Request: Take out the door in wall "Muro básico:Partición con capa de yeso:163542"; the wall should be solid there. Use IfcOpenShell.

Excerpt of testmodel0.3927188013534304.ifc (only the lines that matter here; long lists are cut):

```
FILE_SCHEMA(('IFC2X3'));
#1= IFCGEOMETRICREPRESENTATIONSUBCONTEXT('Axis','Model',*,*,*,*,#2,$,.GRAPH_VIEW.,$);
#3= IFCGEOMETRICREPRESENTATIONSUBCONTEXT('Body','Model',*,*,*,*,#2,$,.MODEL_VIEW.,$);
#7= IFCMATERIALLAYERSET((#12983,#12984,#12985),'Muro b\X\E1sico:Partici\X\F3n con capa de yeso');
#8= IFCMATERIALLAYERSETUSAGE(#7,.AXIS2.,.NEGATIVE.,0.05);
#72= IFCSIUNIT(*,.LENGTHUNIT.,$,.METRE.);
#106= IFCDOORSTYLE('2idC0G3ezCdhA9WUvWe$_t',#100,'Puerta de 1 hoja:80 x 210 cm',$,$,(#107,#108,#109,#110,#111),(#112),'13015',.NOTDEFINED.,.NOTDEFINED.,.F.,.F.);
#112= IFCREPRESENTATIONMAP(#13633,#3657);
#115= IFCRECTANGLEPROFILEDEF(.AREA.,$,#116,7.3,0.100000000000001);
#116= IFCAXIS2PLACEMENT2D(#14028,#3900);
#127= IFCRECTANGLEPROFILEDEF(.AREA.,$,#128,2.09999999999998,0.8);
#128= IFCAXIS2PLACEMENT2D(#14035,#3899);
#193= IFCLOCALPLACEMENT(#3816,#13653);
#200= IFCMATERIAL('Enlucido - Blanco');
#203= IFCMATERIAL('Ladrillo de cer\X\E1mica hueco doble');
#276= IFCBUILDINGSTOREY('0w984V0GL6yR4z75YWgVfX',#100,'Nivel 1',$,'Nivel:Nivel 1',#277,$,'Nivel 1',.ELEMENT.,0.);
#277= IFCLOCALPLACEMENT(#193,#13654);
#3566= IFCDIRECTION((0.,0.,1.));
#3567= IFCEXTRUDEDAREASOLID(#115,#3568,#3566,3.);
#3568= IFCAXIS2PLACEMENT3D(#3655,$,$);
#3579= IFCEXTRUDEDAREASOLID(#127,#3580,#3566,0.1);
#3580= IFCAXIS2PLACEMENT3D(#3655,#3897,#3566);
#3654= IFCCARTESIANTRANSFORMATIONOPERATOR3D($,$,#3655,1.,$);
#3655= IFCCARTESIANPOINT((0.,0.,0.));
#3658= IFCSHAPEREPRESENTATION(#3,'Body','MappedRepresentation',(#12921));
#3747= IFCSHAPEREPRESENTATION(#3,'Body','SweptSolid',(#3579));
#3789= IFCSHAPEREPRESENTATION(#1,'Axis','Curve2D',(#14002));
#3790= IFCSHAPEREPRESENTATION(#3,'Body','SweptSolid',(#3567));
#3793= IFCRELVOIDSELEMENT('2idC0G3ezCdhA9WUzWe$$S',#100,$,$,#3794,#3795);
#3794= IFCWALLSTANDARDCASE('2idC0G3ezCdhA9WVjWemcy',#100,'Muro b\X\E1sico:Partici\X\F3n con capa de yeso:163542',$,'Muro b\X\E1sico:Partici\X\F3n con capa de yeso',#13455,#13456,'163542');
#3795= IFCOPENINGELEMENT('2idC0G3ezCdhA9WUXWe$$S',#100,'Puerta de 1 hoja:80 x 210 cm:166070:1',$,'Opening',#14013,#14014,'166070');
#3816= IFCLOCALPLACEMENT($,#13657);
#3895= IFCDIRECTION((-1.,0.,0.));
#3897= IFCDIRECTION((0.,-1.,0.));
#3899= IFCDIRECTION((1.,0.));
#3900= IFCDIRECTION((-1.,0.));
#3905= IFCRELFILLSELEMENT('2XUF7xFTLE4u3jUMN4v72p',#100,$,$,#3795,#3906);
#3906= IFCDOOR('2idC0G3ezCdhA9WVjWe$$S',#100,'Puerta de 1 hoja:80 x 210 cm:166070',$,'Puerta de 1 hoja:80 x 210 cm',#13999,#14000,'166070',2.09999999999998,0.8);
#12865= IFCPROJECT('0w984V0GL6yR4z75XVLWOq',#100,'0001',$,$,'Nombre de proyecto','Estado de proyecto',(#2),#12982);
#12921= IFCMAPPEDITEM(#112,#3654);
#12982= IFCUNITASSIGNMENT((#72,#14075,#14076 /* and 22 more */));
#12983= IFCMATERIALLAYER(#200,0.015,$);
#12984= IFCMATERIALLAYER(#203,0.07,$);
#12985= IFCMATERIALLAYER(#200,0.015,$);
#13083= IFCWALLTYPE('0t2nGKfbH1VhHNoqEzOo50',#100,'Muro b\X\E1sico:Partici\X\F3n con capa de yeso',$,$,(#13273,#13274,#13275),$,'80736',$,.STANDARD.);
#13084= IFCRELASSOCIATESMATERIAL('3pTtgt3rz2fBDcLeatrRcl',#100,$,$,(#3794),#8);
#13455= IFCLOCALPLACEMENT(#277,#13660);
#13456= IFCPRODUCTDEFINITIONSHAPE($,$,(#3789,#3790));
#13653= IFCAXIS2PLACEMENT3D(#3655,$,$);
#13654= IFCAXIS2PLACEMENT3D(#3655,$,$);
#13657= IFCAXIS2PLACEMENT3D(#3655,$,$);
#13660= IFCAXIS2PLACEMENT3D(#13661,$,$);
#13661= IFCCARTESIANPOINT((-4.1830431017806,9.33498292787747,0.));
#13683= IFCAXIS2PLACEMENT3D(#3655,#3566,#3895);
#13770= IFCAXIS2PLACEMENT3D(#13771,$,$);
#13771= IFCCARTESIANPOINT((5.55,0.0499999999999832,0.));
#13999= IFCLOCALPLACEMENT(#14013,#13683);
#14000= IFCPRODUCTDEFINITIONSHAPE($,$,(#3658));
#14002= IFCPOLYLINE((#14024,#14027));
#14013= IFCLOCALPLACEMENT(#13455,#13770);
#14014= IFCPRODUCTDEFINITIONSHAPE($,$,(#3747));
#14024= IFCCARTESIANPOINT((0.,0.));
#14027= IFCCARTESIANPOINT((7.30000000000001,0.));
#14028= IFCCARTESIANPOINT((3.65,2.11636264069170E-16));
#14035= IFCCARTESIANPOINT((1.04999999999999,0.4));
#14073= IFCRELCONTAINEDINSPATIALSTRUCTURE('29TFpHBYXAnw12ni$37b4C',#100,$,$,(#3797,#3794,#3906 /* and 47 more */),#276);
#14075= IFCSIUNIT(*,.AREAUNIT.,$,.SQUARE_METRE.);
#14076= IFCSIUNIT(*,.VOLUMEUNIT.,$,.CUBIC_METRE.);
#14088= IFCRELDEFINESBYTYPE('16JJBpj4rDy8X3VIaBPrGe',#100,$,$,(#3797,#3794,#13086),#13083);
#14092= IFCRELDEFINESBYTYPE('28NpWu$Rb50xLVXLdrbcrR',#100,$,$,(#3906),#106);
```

```python
import ifcopenshell
import ifcopenshell.api.feature
import ifcopenshell.api.root
import ifcopenshell.geom
import ifcopenshell.util.shape

model = ifcopenshell.open("testmodel0.3927188013534304.ifc")
settings = ifcopenshell.geom.settings()


def volume(element):
    """Net volume in cubic metres, openings subtracted."""
    shape = ifcopenshell.geom.create_shape(settings, element)
    return ifcopenshell.util.shape.get_volume(shape.geometry)


door = model.by_guid("2idC0G3ezCdhA9WVjWe$$S")
opening = door.FillsVoids[0].RelatingOpeningElement
wall = opening.VoidsElements[0].RelatingBuildingElement
before = volume(wall)

ifcopenshell.api.root.remove_product(model, product=door)
ifcopenshell.api.feature.remove_feature(model, feature=opening)

after = volume(wall)

print(f"wall volume {before:.3f} -> {after:.3f} m3")

model.write("testmodel0.3927188013534304_rev.ifc")
```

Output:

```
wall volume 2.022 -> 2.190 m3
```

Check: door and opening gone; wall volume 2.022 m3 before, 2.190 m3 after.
